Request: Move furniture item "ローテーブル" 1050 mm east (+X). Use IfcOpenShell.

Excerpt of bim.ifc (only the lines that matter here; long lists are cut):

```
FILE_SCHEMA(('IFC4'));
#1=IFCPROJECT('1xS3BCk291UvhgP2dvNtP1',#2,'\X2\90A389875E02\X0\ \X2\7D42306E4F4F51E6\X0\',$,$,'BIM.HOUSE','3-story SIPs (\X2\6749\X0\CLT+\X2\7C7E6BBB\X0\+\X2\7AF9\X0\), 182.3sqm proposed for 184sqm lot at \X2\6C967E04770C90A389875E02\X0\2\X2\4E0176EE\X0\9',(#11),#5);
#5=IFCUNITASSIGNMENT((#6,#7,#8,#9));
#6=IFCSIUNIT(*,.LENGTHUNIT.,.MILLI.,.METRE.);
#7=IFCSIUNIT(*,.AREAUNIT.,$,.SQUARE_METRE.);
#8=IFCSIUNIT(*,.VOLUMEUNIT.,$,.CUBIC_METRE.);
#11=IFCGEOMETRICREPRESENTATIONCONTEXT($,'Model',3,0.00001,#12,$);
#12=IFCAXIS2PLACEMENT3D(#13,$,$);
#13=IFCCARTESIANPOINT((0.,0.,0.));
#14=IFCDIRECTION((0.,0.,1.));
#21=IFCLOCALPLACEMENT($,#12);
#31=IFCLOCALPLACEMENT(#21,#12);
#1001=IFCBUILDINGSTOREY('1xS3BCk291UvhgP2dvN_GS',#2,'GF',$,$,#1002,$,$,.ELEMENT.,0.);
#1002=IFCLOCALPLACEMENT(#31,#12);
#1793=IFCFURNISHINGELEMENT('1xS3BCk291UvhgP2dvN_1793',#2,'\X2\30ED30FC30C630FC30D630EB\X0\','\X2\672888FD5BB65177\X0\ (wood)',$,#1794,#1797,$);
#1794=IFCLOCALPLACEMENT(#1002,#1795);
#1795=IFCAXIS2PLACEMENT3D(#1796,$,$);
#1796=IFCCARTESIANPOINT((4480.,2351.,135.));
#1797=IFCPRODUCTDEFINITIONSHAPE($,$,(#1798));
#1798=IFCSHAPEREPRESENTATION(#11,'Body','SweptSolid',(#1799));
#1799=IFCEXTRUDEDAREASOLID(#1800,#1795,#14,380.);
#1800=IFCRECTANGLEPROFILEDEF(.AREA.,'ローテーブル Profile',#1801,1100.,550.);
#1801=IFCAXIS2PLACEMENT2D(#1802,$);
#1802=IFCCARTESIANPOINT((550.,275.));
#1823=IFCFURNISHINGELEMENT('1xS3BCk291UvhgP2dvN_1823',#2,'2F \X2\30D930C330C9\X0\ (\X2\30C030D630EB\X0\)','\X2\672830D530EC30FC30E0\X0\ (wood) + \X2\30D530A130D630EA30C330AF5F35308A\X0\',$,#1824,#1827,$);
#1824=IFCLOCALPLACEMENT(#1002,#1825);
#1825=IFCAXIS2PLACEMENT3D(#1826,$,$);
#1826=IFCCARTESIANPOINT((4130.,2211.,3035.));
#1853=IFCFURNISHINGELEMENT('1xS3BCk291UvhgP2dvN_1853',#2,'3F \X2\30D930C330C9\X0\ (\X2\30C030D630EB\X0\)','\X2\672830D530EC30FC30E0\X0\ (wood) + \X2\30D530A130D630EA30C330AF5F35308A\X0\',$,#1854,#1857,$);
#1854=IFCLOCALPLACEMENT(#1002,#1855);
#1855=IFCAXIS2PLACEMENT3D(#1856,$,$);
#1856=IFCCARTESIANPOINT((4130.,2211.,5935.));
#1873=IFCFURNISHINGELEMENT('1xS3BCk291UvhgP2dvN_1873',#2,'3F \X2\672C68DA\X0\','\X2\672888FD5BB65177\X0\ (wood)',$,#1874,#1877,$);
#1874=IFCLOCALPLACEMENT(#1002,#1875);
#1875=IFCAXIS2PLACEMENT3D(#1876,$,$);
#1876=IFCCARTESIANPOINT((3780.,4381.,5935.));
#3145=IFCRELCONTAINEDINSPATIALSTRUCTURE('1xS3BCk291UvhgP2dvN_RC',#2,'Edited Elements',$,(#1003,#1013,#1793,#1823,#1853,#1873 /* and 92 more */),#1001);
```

```python
import ifcopenshell
import ifcopenshell.api.geometry
import ifcopenshell.util.placement
import ifcopenshell.util.unit

model = ifcopenshell.open("bim.ifc")
unit_scale = ifcopenshell.util.unit.calculate_unit_scale(model)

item = model.by_guid("1xS3BCk291UvhgP2dvN_1793")
matrix = ifcopenshell.util.placement.get_local_placement(item.ObjectPlacement)
matrix[0, 3] += 1.05 / unit_scale
ifcopenshell.api.geometry.edit_object_placement(model, product=item, matrix=matrix, is_si=False)

print(ifcopenshell.util.placement.get_local_placement(item.ObjectPlacement).round(3) + 0.0)

model.write("bim-out.ifc")
```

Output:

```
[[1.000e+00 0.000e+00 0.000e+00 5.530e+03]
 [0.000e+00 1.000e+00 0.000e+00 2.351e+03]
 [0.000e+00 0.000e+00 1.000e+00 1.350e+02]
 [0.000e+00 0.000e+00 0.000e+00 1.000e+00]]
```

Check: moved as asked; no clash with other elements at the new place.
